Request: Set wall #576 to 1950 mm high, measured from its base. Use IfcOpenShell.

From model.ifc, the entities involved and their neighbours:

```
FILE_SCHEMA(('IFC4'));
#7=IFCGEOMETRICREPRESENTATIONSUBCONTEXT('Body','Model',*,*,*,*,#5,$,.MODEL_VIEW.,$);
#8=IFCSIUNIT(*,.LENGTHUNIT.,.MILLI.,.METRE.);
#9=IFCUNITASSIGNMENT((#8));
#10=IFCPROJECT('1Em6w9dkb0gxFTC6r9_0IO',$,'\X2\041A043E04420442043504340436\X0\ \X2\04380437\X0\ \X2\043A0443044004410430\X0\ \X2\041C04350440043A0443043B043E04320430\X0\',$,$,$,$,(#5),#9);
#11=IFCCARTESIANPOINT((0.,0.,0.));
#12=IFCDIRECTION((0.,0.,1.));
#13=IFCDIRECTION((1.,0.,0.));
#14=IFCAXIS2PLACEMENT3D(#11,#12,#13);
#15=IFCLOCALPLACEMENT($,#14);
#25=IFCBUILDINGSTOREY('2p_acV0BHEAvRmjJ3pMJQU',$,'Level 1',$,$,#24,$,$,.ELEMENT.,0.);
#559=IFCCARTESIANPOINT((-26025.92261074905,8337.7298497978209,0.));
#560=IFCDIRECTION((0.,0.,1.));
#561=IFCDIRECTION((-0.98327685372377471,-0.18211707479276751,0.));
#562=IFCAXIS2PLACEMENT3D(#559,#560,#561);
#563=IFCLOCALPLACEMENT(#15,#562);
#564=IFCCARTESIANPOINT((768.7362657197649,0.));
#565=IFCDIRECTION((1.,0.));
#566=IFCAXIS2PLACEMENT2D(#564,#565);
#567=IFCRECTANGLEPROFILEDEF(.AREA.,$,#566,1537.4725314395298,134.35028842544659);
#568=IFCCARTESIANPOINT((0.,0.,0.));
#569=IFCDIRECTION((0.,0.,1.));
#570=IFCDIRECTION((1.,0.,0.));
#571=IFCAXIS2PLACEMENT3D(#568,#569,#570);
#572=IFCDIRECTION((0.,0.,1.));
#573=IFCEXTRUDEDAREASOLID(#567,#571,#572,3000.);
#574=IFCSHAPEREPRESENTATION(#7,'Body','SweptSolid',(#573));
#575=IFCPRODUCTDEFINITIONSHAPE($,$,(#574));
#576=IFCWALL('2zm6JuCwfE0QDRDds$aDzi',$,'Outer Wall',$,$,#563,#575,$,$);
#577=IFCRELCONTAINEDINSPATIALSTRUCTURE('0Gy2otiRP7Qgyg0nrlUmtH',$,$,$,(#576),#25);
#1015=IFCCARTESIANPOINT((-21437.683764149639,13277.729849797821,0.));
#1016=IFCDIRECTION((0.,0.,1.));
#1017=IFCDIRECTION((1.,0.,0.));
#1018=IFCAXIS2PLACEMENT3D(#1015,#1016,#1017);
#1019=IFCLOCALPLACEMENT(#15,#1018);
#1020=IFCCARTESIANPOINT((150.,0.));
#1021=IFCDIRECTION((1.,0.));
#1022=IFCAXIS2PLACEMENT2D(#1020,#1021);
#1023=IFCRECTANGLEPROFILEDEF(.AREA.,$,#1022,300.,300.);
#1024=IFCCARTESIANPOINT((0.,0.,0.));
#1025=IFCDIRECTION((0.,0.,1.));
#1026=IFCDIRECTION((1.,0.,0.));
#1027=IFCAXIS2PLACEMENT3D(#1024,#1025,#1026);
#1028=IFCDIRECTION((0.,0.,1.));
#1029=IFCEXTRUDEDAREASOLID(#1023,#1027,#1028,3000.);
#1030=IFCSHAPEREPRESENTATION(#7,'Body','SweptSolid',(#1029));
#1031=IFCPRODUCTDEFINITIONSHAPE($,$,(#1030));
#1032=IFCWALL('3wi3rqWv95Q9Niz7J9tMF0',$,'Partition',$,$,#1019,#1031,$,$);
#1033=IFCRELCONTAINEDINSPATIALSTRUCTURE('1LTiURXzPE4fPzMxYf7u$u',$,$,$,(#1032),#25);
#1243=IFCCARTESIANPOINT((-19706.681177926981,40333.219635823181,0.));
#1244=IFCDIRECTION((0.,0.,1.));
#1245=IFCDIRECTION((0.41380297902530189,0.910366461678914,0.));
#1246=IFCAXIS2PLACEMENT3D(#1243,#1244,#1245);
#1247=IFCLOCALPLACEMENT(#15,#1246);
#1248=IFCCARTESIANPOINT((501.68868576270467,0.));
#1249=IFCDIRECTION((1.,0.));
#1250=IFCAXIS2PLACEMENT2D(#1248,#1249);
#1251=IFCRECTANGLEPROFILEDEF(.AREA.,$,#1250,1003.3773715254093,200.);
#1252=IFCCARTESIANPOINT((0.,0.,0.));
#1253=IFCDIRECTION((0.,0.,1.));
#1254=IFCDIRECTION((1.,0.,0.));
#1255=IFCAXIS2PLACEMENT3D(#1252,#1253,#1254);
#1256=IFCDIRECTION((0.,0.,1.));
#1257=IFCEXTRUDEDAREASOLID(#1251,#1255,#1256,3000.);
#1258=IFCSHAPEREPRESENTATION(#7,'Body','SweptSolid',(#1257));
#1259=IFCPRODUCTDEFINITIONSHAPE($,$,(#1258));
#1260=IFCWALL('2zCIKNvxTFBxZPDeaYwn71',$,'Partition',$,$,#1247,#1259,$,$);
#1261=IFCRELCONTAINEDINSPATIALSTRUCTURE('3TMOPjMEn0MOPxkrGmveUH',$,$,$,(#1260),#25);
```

```python
import ifcopenshell
import ifcopenshell.geom
import ifcopenshell.util.representation
import ifcopenshell.util.shape

model = ifcopenshell.open("model.ifc")
settings = ifcopenshell.geom.settings()


def volume(element):
    """Net volume in cubic metres, openings subtracted."""
    shape = ifcopenshell.geom.create_shape(settings, element)
    return ifcopenshell.util.shape.get_volume(shape.geometry)


wall = model.by_guid("2zm6JuCwfE0QDRDds$aDzi")
before = volume(wall)

body = ifcopenshell.util.representation.get_representation(wall, "Model", "Body")
solid = body.Items[0]
old_height = solid.Depth
solid.Depth = 1950.0
after = volume(wall)

print(f"height {old_height:g} -> {solid.Depth:g}, volume {before:.3f} -> {after:.3f} m3")

model.write("model-out.ifc")
```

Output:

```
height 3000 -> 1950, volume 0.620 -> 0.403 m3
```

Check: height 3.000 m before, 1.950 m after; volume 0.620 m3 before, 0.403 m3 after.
